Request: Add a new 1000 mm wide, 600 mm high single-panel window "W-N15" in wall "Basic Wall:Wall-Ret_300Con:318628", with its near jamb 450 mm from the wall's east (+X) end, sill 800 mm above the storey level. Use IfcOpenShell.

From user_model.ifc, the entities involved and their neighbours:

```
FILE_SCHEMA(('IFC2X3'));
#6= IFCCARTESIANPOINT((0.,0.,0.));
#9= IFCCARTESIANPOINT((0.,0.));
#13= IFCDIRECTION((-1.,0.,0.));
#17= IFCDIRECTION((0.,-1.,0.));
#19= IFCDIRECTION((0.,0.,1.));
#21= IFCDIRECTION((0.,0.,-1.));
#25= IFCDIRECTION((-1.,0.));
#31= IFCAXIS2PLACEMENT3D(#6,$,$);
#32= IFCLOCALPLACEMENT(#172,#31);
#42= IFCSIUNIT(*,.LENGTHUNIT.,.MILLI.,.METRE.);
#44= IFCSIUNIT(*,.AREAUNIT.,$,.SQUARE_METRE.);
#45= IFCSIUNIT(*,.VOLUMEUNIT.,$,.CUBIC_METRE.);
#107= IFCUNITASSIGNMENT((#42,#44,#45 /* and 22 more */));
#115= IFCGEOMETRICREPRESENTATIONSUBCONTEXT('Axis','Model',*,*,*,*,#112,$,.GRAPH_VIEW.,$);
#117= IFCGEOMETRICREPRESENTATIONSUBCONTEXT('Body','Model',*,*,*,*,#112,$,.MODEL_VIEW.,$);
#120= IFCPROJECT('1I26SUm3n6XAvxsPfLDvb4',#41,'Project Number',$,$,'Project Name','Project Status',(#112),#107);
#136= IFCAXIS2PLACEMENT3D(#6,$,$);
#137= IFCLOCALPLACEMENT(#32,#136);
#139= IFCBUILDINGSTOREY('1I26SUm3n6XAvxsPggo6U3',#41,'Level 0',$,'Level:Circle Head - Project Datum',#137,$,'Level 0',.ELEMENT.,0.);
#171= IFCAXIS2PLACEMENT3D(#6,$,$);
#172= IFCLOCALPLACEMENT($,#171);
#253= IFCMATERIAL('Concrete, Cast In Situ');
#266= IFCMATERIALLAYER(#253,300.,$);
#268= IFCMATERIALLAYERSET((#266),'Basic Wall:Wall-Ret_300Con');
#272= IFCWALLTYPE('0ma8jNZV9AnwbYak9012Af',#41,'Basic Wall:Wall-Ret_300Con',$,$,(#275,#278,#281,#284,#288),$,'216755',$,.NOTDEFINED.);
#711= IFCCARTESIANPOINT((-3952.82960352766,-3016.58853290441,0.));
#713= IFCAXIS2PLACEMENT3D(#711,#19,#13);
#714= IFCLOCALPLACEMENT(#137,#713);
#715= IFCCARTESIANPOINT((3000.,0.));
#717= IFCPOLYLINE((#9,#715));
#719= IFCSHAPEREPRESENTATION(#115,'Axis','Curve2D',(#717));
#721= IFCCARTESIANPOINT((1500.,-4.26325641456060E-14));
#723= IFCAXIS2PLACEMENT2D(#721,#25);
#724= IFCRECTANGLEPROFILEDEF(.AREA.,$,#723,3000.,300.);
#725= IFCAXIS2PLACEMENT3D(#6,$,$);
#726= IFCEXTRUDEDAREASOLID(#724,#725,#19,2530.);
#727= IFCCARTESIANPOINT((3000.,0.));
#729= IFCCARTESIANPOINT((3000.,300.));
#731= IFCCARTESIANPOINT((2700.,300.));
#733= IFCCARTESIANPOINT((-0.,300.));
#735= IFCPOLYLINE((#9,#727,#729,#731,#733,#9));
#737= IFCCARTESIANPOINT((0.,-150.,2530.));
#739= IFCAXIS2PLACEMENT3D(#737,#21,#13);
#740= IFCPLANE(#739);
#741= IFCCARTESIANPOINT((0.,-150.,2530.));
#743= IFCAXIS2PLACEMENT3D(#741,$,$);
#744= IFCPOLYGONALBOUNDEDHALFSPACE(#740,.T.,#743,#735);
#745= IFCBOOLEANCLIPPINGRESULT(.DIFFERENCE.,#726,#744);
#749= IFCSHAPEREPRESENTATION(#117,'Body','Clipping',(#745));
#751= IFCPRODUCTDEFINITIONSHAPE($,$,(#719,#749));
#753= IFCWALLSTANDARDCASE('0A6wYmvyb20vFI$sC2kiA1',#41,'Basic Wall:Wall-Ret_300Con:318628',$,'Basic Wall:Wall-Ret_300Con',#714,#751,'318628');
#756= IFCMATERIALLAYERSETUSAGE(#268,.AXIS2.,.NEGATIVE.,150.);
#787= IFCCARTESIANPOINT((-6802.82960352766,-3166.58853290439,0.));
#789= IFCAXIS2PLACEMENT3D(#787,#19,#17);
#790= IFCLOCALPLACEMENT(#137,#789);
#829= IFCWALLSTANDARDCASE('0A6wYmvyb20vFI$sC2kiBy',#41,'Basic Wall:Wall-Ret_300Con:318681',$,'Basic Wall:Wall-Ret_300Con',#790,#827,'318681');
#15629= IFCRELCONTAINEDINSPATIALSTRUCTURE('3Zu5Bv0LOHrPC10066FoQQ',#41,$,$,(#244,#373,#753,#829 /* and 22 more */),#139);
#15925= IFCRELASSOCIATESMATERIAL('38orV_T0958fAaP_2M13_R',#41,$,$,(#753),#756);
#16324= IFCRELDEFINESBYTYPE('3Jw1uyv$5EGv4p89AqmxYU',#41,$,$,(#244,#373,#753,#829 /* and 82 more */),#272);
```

```python
import numpy as np
import ifcopenshell
import ifcopenshell.api.feature
import ifcopenshell.api.geometry
import ifcopenshell.api.root
import ifcopenshell.api.spatial
import ifcopenshell.api.type
import ifcopenshell.geom
import ifcopenshell.util.element
import ifcopenshell.util.placement
import ifcopenshell.util.representation
import ifcopenshell.util.shape
import ifcopenshell.util.unit

model = ifcopenshell.open("user_model.ifc")
unit_scale = ifcopenshell.util.unit.calculate_unit_scale(model)
settings = ifcopenshell.geom.settings()


def volume(element):
    """Net volume in cubic metres, openings subtracted."""
    shape = ifcopenshell.geom.create_shape(settings, element)
    return ifcopenshell.util.shape.get_volume(shape.geometry)


wall = model.by_guid("0A6wYmvyb20vFI$sC2kiA1")
storey = ifcopenshell.util.element.get_container(wall, ifc_class="IfcBuildingStorey")
context = ifcopenshell.util.representation.get_context(model, "Model", "Body", "MODEL_VIEW")
before = volume(wall)

width, height, from_end, sill = 1, 0.6, 0.45, 0.8  # metres

# The wall runs along its own X axis, and the end named is its -X end.
wall_shape = ifcopenshell.geom.create_shape(settings, wall)
x, y, z = ifcopenshell.util.shape.get_vertices(wall_shape.geometry).T
start = x.min() + from_end
face, thickness = float(y.min()), float(y.max() - y.min())
wall_matrix = ifcopenshell.util.placement.get_local_placement(wall.ObjectPlacement)
level = ifcopenshell.util.placement.get_local_placement(storey.ObjectPlacement)[2, 3]


def in_wall(x, y):
    """Placement at x, y metres in the wall's axes, at sill height."""
    matrix = wall_matrix.copy()
    matrix[:, 3] = wall_matrix @ np.array([x / unit_scale, y / unit_scale, 0.0, 1.0])
    matrix[2, 3] = level + sill / unit_scale
    return matrix


# Opening: a box that overshoots both wall faces by 50 mm.
opening = ifcopenshell.api.root.create_entity(model, ifc_class="IfcOpeningElement")
box = ifcopenshell.api.geometry.add_wall_representation(
    model, context=context, length=width, height=height, thickness=thickness + 0.1
)
ifcopenshell.api.geometry.assign_representation(model, product=opening, representation=box)
ifcopenshell.api.geometry.edit_object_placement(model, product=opening, matrix=in_wall(start, face - 0.05), is_si=False)
ifcopenshell.api.feature.add_feature(model, feature=opening, element=wall)

window = ifcopenshell.api.root.create_entity(model, ifc_class="IfcWindow", name="W-N15")
window.OverallWidth, window.OverallHeight = width / unit_scale, height / unit_scale
body = ifcopenshell.api.geometry.add_window_representation(
    model,
    context=context,
    overall_width=window.OverallWidth,
    overall_height=window.OverallHeight,
    partition_type="SINGLE_PANEL",
)
ifcopenshell.api.geometry.assign_representation(model, product=window, representation=body)
ifcopenshell.api.spatial.assign_container(model, products=[window], relating_structure=storey)
fills = ifcopenshell.api.feature.add_filling(model, opening=opening, element=window)
fills.OwnerHistory = window.OwnerHistory  # required in IFC2X3

# IFC2X3 keeps the operation on the window style.
style = ifcopenshell.api.root.create_entity(model, ifc_class="IfcWindowStyle", name="W-N15")
style.OperationType, style.ConstructionType = "SINGLE_PANEL", "NOTDEFINED"
style.ParameterTakesPrecedence = style.Sizeable = False
ifcopenshell.api.type.assign_type(model, related_objects=[window], relating_type=style)

# Centre the window in the wall's thickness.
ifcopenshell.api.geometry.edit_object_placement(model, product=window, matrix=in_wall(start, face), is_si=False)
window_shape = ifcopenshell.geom.create_shape(settings, window)
depth = ifcopenshell.util.shape.get_vertices(window_shape.geometry)[:, 1]
offset = face + thickness / 2 - (depth.min() + depth.max()) / 2
ifcopenshell.api.geometry.edit_object_placement(model, product=window, matrix=in_wall(start, offset), is_si=False)

after = volume(wall)

print(f"wall volume {before:.3f} -> {after:.3f} m3")

model.write("user_model_updated.ifc")
```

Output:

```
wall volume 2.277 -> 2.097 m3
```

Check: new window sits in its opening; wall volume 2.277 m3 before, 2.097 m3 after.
